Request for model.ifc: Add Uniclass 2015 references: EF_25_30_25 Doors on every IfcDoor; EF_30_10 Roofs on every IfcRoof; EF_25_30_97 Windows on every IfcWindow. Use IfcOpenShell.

First a look at what the model holds.

```python
import ifcopenshell

model = ifcopenshell.open("model.ifc")
print(model.schema)
print("classifications:", [c.Name for c in model.by_type("IfcClassification")])
for ifc_class in ("IfcDoor", "IfcRoof", "IfcStair", "IfcWall", "IfcWindow"):
    print(ifc_class, len(model.by_type(ifc_class)))
```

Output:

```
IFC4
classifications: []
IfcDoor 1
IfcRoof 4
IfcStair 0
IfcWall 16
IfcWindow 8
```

```python
import ifcopenshell
import ifcopenshell.api.classification

model = ifcopenshell.open("model.ifc")

system = ifcopenshell.api.classification.add_classification(model, classification="Uniclass 2015")

codes = {
    "IfcDoor": ("EF_25_30_25", "Doors"),
    "IfcRoof": ("EF_30_10", "Roofs"),
    "IfcWindow": ("EF_25_30_97", "Windows"),
}
for ifc_class, (code, name) in codes.items():
    products = model.by_type(ifc_class)
    ifcopenshell.api.classification.add_reference(
        model, products=products, classification=system, identification=code, name=name
    )
    print(code, len(products))

model.write("model_v2.ifc")
```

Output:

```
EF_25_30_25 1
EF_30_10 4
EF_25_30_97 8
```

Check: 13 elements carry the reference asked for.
